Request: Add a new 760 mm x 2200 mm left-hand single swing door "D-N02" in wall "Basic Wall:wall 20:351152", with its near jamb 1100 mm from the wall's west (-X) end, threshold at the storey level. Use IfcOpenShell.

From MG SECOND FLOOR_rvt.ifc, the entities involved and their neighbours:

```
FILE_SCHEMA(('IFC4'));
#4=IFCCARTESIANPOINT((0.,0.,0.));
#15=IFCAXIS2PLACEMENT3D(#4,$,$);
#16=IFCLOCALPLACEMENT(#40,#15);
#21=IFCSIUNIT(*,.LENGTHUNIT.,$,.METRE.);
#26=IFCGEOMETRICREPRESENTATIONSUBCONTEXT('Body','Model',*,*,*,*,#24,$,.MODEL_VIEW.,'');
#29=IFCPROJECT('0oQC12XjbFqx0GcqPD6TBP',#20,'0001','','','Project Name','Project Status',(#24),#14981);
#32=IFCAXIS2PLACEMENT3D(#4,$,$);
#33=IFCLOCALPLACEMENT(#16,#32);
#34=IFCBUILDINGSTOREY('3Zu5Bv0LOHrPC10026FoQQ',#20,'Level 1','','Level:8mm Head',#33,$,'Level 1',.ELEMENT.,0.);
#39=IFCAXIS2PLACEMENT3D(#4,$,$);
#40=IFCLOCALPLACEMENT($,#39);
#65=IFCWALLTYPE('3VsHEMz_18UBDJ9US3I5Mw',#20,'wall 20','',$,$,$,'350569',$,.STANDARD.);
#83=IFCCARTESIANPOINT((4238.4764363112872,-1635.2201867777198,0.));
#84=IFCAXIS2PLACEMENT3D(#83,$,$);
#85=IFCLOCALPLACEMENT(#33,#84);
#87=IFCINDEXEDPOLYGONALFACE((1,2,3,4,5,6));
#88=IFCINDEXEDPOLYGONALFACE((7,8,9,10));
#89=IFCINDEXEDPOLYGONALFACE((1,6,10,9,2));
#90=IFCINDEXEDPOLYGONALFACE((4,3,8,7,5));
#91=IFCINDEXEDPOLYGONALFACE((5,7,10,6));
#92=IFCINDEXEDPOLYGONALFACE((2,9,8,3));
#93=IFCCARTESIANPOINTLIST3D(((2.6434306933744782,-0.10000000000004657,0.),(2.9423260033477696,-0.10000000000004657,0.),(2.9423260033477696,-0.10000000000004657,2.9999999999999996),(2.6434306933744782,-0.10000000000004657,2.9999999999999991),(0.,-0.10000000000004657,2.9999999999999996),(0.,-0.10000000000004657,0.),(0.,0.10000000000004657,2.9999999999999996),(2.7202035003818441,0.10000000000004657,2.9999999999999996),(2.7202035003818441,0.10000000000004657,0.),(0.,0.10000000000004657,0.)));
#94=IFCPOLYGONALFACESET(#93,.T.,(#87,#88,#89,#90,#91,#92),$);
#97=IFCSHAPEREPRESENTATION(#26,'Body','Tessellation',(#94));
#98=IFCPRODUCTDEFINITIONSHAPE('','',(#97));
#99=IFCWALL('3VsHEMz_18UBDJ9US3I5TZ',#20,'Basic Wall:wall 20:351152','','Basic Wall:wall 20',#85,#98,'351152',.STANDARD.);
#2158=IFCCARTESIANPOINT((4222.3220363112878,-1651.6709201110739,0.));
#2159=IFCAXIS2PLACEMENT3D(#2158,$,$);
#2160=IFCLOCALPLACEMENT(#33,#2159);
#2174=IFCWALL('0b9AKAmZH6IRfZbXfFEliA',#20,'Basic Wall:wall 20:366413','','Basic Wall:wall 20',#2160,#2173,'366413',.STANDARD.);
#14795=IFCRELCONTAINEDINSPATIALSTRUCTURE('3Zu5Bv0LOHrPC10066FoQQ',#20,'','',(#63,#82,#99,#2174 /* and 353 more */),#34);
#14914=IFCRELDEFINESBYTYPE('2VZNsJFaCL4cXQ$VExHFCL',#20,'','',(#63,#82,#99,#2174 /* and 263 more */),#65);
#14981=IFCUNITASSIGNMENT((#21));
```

```python
import numpy as np
import ifcopenshell
import ifcopenshell.api.feature
import ifcopenshell.api.geometry
import ifcopenshell.api.root
import ifcopenshell.api.spatial
import ifcopenshell.geom
import ifcopenshell.util.element
import ifcopenshell.util.placement
import ifcopenshell.util.representation
import ifcopenshell.util.shape
import ifcopenshell.util.unit

model = ifcopenshell.open("MG SECOND FLOOR_rvt.ifc")
unit_scale = ifcopenshell.util.unit.calculate_unit_scale(model)
settings = ifcopenshell.geom.settings()


def volume(element):
    """Net volume in cubic metres, openings subtracted."""
    shape = ifcopenshell.geom.create_shape(settings, element)
    return ifcopenshell.util.shape.get_volume(shape.geometry)


wall = model.by_guid("3VsHEMz_18UBDJ9US3I5TZ")
storey = ifcopenshell.util.element.get_container(wall, ifc_class="IfcBuildingStorey")
context = ifcopenshell.util.representation.get_context(model, "Model", "Body", "MODEL_VIEW")
before = volume(wall)

width, height, from_end, sill = 0.76, 2.2, 1.1, 0.0  # metres

# The wall runs along its own X axis, and the end named is its -X end.
wall_shape = ifcopenshell.geom.create_shape(settings, wall)
x, y, z = ifcopenshell.util.shape.get_vertices(wall_shape.geometry).T
start = x.min() + from_end
face, thickness = float(y.min()), float(y.max() - y.min())
wall_matrix = ifcopenshell.util.placement.get_local_placement(wall.ObjectPlacement)
level = ifcopenshell.util.placement.get_local_placement(storey.ObjectPlacement)[2, 3]


def in_wall(x, y):
    """Placement at x, y metres in the wall's axes, at sill height."""
    matrix = wall_matrix.copy()
    matrix[:, 3] = wall_matrix @ np.array([x / unit_scale, y / unit_scale, 0.0, 1.0])
    matrix[2, 3] = level + sill / unit_scale
    return matrix


# Opening: a box that overshoots both wall faces by 50 mm.
opening = ifcopenshell.api.root.create_entity(model, ifc_class="IfcOpeningElement", predefined_type="OPENING")
box = ifcopenshell.api.geometry.add_wall_representation(
    model, context=context, length=width, height=height, thickness=thickness + 0.1
)
ifcopenshell.api.geometry.assign_representation(model, product=opening, representation=box)
ifcopenshell.api.geometry.edit_object_placement(model, product=opening, matrix=in_wall(start, face - 0.05), is_si=False)
ifcopenshell.api.feature.add_feature(model, feature=opening, element=wall)

door = ifcopenshell.api.root.create_entity(model, ifc_class="IfcDoor", name="D-N02", predefined_type="DOOR")
door.OverallWidth, door.OverallHeight = width / unit_scale, height / unit_scale
door.OperationType = "SINGLE_SWING_LEFT"
body = ifcopenshell.api.geometry.add_door_representation(
    model,
    context=context,
    overall_width=door.OverallWidth,
    overall_height=door.OverallHeight,
    operation_type="SINGLE_SWING_LEFT",
    lining_properties={"LiningDepth": thickness / unit_scale, "ThresholdDepth": thickness / unit_scale},
)
ifcopenshell.api.geometry.assign_representation(model, product=door, representation=body)
ifcopenshell.api.spatial.assign_container(model, products=[door], relating_structure=storey)
ifcopenshell.api.feature.add_filling(model, opening=opening, element=door)

# The lining spans the wall, so the door starts at the wall face.
ifcopenshell.api.geometry.edit_object_placement(model, product=door, matrix=in_wall(start, face), is_si=False)

after = volume(wall)

print(f"wall volume {before:.3f} -> {after:.3f} m3")

model.write("MG SECOND FLOOR_rvt_updated.ifc")
```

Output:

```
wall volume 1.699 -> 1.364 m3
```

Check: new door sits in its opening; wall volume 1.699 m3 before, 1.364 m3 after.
